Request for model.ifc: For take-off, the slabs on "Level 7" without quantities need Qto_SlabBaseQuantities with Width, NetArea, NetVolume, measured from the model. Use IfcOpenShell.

First a look at what the model holds.

```python
import ifcopenshell
import ifcopenshell.util.element
import ifcopenshell.util.unit

model = ifcopenshell.open("model.ifc")
print(model.schema)
for unit_type in ("LENGTHUNIT", "AREAUNIT", "VOLUMEUNIT"):
    print(unit_type, ifcopenshell.util.unit.calculate_unit_scale(model, unit_type))
storey = next(s for s in model.by_type("IfcBuildingStorey") if s.Name == "Level 7")
slabs = [e for e in ifcopenshell.util.element.get_decomposition(storey) if e.is_a("IfcSlab")]
for e in sorted(slabs, key=lambda e: e.id()):
    print(e.id(), e.is_a(), e.Name, list(ifcopenshell.util.element.get_psets(e, qtos_only=True)), sep=" | ")
```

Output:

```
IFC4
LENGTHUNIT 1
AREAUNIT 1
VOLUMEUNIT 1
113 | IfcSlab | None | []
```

```python
import ifcopenshell
import ifcopenshell.api.pset
import ifcopenshell.geom
import ifcopenshell.util.element
import ifcopenshell.util.shape
import ifcopenshell.util.unit

model = ifcopenshell.open("model.ifc")
unit_scale = ifcopenshell.util.unit.calculate_unit_scale(model)
area_scale = ifcopenshell.util.unit.calculate_unit_scale(model, "AREAUNIT")
volume_scale = ifcopenshell.util.unit.calculate_unit_scale(model, "VOLUMEUNIT")
settings = ifcopenshell.geom.settings()

storey = next(s for s in model.by_type("IfcBuildingStorey") if s.Name == "Level 7")
slabs = [e for e in ifcopenshell.util.element.get_decomposition(storey) if e.is_a("IfcSlab")]

for e in sorted(slabs, key=lambda e: e.id()):
    if ifcopenshell.util.element.get_psets(e, qtos_only=True, should_inherit=False):
        continue
    # Geometry comes back in metres, in the element's own axes.
    shape = ifcopenshell.geom.create_shape(settings, e)
    values = {
        "Width": ifcopenshell.util.shape.get_z(shape.geometry) / unit_scale,
        "NetArea": ifcopenshell.util.shape.get_footprint_area(shape.geometry) / area_scale,
        "NetVolume": ifcopenshell.util.shape.get_volume(shape.geometry) / volume_scale,
    }
    qto = ifcopenshell.api.pset.add_qto(model, product=e, name="Qto_SlabBaseQuantities")
    ifcopenshell.api.pset.edit_qto(model, qto=qto, properties=values)
    print(e.id(), {k: round(v, 3) for k, v in values.items()})

model.write("model_edited.ifc")
```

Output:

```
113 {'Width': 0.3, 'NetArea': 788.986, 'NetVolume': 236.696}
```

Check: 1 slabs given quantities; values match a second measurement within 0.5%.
